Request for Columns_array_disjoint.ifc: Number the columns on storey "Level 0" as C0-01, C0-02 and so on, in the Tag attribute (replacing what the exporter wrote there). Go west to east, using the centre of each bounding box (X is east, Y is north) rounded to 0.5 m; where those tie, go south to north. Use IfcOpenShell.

First a look at what the model holds.

```python
import ifcopenshell
import ifcopenshell.util.element
import ifcopenshell.util.placement

model = ifcopenshell.open("Columns_array_disjoint.ifc")
print(model.schema)
storey = next(s for s in model.by_type("IfcBuildingStorey") if s.Name == "Level 0")
columns = [e for e in ifcopenshell.util.element.get_decomposition(storey) if e.is_a("IfcColumn")]
for e in sorted(columns, key=lambda e: e.id()):
    origin = ifcopenshell.util.placement.get_local_placement(e.ObjectPlacement)[:3, 3]
    print(e.id(), e.Tag, e.Name, origin.round(2) + 0.0, sep=" | ")
```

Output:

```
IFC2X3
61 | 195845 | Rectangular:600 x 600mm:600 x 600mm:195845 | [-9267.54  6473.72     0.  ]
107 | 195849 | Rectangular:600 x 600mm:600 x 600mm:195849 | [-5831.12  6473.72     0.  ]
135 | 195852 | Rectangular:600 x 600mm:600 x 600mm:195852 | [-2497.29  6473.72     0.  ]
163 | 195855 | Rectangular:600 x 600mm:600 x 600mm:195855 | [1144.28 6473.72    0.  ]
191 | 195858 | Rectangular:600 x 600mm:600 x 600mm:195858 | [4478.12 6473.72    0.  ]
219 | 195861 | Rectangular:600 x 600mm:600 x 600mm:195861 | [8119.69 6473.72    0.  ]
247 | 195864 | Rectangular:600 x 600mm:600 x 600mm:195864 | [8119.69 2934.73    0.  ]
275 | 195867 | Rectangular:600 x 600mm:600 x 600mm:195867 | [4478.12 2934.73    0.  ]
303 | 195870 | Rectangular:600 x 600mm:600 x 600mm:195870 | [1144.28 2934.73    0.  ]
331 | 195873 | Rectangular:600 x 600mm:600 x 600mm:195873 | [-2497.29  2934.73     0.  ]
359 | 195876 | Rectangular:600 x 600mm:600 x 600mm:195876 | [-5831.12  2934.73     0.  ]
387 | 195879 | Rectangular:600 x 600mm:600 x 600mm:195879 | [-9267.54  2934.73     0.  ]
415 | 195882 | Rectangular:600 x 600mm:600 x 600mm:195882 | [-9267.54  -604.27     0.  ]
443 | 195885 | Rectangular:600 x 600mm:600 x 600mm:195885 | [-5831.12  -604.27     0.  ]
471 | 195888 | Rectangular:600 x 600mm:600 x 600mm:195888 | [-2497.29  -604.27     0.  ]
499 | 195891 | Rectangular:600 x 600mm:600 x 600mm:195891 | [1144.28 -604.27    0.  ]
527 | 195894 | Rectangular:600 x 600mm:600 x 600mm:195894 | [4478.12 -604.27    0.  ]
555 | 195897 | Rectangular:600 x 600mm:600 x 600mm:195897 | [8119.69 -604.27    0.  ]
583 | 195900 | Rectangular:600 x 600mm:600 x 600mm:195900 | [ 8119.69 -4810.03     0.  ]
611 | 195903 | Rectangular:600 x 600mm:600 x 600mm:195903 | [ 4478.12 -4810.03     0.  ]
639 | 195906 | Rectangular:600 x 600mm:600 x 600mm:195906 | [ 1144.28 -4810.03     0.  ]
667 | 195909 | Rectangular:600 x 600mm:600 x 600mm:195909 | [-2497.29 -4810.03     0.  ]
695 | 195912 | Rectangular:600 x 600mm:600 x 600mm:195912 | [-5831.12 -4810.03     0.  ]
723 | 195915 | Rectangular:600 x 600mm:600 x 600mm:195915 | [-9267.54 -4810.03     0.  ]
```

```python
import ifcopenshell
import ifcopenshell.geom
import ifcopenshell.util.element
import ifcopenshell.util.shape

model = ifcopenshell.open("Columns_array_disjoint.ifc")
settings = ifcopenshell.geom.settings()
settings.set("use-world-coords", True)


def centre(element):
    shape = ifcopenshell.geom.create_shape(settings, element)
    return ifcopenshell.util.shape.get_bbox_centroid(shape.geometry)


storey = next(s for s in model.by_type("IfcBuildingStorey") if s.Name == "Level 0")
columns = [e for e in ifcopenshell.util.element.get_decomposition(storey) if e.is_a("IfcColumn")]

# Insertion points can sit at a corner or the storey origin, so sort by the geometry (in metres).
centres = {e: centre(e) for e in columns}
columns.sort(key=lambda e: (round(centres[e][0] / 0.5), centres[e][1]))

for i, e in enumerate(columns, start=1):
    number = f"C0-{i:02d}"
    e.Tag = number
    print(e.id(), number)

model.write("Columns_array_disjoint-out.ifc")
```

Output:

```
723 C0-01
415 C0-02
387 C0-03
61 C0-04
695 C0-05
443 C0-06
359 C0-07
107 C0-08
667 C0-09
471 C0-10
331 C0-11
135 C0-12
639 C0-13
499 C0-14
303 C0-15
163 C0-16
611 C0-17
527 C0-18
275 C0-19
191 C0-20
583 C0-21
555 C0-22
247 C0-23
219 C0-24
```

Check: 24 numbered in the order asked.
